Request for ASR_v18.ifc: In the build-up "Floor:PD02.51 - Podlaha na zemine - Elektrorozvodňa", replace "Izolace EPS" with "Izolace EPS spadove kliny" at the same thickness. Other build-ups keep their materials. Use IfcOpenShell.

First a look at what the model holds.

```python
import ifcopenshell
import ifcopenshell.util.element

model = ifcopenshell.open("ASR_v18.ifc")
print(model.schema)
for layer_set in model.by_type("IfcMaterialLayerSet"):
    if layer_set.LayerSetName == "Floor:PD02.51 - Podlaha na zemine - Elektrorozvodňa":
        for layer in layer_set.MaterialLayers:
            print(layer.id(), layer.Material and layer.Material.Name, layer.LayerThickness, sep=" | ")
        print(len(ifcopenshell.util.element.get_elements_by_material(model, layer_set)), "elements and types use it")
print(sorted(m.Name for m in model.by_type("IfcMaterial") if m.Name)[:60])
```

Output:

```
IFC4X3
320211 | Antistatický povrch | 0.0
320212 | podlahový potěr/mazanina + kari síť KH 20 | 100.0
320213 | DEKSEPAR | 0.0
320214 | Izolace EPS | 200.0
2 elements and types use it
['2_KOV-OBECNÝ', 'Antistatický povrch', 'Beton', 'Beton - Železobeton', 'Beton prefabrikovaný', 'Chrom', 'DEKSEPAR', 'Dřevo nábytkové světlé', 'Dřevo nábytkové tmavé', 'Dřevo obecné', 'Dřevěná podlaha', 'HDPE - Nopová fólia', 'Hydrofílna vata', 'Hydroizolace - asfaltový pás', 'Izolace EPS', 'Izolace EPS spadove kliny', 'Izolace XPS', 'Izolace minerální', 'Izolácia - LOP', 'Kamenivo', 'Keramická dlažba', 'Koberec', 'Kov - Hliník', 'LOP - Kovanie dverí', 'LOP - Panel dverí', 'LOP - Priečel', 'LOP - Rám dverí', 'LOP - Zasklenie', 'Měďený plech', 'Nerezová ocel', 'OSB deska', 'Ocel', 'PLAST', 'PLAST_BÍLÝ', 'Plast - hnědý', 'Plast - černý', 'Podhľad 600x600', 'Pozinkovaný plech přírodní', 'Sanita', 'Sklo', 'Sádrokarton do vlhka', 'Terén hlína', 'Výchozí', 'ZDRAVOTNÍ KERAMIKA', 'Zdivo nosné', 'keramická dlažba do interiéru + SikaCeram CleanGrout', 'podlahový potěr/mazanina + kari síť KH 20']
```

```python
import ifcopenshell
import ifcopenshell.api.material

model = ifcopenshell.open("ASR_v18.ifc")

layer_set = next(s for s in model.by_type("IfcMaterialLayerSet") if s.LayerSetName == "Floor:PD02.51 - Podlaha na zemine - Elektrorozvodňa")
layer = next(l for l in layer_set.MaterialLayers if l.Material and l.Material.Name == "Izolace EPS")
material = next(m for m in model.by_type("IfcMaterial") if m.Name == "Izolace EPS spadove kliny")

# Point this one layer at the other material; renaming the old one would change it everywhere.
ifcopenshell.api.material.edit_layer(model, layer=layer, attributes={"Name": material.Name}, material=material)

print([l.Material.Name if l.Material else None for l in layer_set.MaterialLayers])

model.write("ASR_v18_v2.ifc")
```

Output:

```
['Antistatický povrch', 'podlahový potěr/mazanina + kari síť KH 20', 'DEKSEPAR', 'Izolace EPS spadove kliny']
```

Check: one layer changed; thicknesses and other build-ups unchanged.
